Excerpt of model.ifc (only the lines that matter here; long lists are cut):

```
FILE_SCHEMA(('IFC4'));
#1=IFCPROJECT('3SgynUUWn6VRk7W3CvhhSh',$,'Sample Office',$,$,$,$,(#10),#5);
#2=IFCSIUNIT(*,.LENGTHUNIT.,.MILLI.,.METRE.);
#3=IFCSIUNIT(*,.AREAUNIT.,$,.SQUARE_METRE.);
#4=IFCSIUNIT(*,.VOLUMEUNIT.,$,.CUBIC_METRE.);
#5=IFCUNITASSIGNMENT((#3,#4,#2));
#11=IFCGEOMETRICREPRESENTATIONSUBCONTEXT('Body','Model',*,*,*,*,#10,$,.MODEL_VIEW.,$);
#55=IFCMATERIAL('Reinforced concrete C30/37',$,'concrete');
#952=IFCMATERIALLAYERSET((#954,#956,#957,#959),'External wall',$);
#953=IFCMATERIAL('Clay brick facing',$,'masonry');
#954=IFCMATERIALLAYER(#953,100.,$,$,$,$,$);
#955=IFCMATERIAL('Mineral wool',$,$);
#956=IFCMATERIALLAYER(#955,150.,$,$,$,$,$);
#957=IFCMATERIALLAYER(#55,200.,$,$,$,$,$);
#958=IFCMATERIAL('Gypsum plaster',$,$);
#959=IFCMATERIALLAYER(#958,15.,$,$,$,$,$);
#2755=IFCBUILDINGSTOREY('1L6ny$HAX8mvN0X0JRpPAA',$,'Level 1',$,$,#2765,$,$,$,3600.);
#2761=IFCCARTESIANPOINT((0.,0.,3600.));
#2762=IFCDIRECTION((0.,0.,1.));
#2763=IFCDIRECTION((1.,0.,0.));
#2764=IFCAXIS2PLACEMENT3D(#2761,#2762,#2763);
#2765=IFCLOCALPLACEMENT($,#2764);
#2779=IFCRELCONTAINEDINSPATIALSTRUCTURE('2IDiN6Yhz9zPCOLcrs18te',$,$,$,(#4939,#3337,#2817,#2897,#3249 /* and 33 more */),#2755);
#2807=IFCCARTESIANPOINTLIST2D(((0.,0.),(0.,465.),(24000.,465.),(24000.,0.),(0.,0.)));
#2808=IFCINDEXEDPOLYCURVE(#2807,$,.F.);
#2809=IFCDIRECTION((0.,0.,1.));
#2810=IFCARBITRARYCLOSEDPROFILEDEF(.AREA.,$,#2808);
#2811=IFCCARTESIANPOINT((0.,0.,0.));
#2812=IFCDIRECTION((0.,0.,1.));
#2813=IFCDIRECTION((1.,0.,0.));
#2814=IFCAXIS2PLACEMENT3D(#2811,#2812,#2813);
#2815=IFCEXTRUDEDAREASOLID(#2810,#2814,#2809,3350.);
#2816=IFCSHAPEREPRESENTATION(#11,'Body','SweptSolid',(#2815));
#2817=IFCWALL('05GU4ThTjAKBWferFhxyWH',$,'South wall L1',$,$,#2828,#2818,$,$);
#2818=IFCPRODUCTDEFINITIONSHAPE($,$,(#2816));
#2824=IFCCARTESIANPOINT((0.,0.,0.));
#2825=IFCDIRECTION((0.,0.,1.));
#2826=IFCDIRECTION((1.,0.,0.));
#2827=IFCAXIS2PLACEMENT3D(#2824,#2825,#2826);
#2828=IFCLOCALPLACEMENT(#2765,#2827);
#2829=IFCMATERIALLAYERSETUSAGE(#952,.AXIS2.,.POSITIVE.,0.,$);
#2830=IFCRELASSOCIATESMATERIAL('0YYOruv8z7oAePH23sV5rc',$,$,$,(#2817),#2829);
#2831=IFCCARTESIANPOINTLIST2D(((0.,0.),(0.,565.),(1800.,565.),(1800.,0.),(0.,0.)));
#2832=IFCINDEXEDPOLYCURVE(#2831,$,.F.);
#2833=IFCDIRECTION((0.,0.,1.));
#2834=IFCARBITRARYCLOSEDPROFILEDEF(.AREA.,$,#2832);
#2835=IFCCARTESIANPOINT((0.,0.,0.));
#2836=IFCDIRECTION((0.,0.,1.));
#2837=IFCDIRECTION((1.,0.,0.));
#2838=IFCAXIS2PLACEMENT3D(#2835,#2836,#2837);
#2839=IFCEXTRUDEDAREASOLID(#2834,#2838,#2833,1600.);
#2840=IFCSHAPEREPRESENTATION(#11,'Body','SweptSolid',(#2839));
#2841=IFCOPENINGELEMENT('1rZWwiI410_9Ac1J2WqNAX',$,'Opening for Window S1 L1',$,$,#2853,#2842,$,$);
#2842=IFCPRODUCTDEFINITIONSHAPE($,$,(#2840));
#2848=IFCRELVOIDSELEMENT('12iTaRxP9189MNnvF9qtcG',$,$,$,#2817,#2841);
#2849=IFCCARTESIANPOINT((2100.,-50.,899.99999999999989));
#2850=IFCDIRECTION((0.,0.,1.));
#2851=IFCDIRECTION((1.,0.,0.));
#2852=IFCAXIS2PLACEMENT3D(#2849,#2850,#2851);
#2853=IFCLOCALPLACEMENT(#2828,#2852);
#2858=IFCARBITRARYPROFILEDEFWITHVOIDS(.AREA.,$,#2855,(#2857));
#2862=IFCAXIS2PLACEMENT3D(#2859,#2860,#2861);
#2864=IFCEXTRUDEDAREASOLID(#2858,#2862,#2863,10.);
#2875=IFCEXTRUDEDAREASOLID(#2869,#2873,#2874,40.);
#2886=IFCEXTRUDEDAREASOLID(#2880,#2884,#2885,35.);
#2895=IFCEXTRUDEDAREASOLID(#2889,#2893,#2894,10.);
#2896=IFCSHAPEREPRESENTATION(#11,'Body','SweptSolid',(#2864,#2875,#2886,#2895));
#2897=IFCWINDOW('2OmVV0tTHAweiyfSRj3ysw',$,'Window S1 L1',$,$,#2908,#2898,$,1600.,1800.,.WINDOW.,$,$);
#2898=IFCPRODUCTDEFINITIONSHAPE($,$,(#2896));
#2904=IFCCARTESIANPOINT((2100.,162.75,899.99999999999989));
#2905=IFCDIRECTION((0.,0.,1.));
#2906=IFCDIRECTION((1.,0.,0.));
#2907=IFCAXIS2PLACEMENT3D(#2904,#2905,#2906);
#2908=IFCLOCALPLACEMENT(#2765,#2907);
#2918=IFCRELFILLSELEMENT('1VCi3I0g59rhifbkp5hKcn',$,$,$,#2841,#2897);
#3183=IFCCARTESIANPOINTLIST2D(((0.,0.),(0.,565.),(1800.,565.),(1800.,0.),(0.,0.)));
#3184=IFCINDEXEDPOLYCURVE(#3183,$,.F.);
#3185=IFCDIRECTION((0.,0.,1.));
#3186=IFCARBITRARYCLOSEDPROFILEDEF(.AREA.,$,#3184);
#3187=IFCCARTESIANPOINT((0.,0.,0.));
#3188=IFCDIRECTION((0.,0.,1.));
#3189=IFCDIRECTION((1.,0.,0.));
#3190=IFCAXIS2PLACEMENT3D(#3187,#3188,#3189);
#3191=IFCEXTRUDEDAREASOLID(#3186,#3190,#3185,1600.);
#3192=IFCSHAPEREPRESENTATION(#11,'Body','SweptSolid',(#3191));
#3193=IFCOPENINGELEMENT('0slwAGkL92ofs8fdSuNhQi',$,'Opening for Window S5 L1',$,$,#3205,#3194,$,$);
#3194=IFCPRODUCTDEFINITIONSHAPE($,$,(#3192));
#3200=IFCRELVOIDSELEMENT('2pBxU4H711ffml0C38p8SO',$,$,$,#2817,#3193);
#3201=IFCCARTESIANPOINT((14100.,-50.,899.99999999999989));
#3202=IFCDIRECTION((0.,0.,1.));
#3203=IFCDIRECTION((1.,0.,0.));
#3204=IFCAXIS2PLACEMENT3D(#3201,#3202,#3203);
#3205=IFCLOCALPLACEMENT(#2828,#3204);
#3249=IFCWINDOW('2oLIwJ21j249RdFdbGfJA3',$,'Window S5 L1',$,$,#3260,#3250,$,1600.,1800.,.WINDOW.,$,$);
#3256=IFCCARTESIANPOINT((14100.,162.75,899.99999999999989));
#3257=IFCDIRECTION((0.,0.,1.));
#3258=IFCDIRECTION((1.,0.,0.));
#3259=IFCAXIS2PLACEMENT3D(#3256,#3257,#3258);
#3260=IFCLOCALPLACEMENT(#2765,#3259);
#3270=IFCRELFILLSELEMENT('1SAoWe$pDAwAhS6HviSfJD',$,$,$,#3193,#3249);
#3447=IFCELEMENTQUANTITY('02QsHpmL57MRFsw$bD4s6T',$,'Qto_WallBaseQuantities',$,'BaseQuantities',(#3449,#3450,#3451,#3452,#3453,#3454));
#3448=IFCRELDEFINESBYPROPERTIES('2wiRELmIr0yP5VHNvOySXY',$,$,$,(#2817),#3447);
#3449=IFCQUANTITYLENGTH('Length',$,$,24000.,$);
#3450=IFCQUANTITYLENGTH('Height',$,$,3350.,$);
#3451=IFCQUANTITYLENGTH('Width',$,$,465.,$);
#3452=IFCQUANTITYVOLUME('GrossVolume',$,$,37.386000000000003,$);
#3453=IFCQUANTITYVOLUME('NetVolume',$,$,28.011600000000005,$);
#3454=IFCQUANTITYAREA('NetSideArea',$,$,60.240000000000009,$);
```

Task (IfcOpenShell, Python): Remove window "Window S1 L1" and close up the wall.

```python
import ifcopenshell
import ifcopenshell.api.feature
import ifcopenshell.api.pset
import ifcopenshell.api.root
import ifcopenshell.geom
import ifcopenshell.util.element
import ifcopenshell.util.shape
import ifcopenshell.util.unit

model = ifcopenshell.open("model.ifc")
area_scale = ifcopenshell.util.unit.calculate_unit_scale(model, "AREAUNIT")
volume_scale = ifcopenshell.util.unit.calculate_unit_scale(model, "VOLUMEUNIT")
settings = ifcopenshell.geom.settings()


def volume(element):
    """Net volume in cubic metres, openings subtracted."""
    shape = ifcopenshell.geom.create_shape(settings, element)
    return ifcopenshell.util.shape.get_volume(shape.geometry)


window = model.by_guid("2OmVV0tTHAweiyfSRj3ysw")
opening = window.FillsVoids[0].RelatingOpeningElement
wall = opening.VoidsElements[0].RelatingBuildingElement
before = volume(wall)

ifcopenshell.api.root.remove_product(model, product=window)
ifcopenshell.api.feature.remove_feature(model, feature=opening)

after = volume(wall)
thickness = 0.465  # wall thickness in metres

# Update the wall's stored quantities.
qto = model.by_id(ifcopenshell.util.element.get_pset(wall, "Qto_WallBaseQuantities", should_inherit=False)["id"])
ifcopenshell.api.pset.edit_qto(model, qto=qto, properties={
    "NetVolume": after / volume_scale,
    "NetSideArea": after / thickness / area_scale,
})

print(f"wall volume {before:.3f} -> {after:.3f} m3")

model.write("model_updated.ifc")
```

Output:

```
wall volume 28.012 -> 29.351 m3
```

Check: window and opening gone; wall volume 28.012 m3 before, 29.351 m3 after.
